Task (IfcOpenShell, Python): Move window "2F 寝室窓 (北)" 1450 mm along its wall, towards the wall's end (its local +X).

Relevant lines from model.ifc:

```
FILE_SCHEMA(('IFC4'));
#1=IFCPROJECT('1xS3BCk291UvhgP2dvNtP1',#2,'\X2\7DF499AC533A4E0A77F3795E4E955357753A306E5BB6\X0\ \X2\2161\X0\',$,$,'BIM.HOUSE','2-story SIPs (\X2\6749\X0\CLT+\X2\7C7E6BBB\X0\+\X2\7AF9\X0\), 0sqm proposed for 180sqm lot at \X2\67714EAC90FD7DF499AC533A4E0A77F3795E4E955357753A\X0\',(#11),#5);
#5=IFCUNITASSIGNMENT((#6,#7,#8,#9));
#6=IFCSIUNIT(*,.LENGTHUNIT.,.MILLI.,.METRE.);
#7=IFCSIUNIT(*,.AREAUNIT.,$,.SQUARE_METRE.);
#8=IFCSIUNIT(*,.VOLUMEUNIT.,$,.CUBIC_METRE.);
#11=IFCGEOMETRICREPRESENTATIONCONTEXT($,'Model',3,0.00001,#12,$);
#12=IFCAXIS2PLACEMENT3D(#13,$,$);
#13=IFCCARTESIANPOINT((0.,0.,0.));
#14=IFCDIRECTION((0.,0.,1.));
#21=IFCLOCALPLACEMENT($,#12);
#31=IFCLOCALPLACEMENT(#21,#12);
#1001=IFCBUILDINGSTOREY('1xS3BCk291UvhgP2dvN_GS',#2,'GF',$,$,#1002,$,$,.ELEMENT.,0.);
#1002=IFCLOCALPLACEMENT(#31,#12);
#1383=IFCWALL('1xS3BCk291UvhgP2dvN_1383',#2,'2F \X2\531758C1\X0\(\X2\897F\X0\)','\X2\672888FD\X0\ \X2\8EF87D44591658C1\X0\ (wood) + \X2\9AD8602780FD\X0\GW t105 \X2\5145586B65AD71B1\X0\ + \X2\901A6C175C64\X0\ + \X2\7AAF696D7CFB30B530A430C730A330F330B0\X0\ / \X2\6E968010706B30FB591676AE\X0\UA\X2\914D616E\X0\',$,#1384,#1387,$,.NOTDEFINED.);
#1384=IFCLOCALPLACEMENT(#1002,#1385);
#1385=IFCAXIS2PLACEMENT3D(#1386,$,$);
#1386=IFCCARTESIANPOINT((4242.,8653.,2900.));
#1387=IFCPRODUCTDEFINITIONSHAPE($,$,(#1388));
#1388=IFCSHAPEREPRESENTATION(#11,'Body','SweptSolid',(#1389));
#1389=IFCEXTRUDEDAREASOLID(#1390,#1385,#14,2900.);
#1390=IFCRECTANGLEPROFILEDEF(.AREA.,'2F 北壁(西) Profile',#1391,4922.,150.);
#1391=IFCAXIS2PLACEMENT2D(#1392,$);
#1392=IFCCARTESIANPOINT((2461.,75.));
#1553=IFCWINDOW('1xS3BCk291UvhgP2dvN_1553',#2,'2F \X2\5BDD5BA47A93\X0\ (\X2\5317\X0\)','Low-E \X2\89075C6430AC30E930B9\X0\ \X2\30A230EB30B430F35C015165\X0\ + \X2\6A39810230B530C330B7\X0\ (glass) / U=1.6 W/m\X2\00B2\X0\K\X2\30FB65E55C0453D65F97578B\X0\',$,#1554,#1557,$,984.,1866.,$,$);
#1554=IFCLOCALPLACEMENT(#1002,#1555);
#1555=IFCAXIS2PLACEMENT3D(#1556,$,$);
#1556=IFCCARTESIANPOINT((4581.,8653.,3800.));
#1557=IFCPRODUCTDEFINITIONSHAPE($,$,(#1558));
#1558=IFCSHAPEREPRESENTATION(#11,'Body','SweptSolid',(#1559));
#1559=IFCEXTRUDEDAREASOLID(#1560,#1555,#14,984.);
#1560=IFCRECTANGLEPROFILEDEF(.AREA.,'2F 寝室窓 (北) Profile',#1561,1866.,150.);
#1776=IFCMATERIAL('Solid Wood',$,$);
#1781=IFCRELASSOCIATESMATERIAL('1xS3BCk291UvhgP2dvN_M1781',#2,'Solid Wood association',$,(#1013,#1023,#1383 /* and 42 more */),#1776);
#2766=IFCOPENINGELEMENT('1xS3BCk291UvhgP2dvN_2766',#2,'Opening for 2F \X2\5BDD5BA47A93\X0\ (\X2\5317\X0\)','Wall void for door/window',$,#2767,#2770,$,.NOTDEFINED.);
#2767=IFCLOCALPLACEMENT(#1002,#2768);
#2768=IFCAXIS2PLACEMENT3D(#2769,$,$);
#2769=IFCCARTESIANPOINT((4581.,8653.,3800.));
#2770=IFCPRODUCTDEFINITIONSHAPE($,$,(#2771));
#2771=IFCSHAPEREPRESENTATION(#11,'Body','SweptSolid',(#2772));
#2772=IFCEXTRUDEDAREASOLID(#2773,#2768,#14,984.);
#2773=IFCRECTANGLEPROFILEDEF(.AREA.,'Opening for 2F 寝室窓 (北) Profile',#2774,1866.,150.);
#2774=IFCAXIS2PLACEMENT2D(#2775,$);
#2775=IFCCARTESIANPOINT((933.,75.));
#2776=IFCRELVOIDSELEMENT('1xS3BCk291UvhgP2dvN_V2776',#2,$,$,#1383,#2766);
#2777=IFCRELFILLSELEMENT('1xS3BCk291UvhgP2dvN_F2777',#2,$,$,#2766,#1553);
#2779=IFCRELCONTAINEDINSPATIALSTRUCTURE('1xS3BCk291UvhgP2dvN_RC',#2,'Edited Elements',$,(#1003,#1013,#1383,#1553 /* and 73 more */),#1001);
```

```python
import ifcopenshell
import ifcopenshell.api.geometry
import ifcopenshell.util.placement

model = ifcopenshell.open("model.ifc")

window = model.by_guid("1xS3BCk291UvhgP2dvN_1553")
opening = window.FillsVoids[0].RelatingOpeningElement
wall = opening.VoidsElements[0].RelatingBuildingElement

wall_matrix = ifcopenshell.util.placement.get_local_placement(wall.ObjectPlacement)
shift = wall_matrix[:3, 0] * 1450.0
before = ifcopenshell.util.placement.get_local_placement(window.ObjectPlacement)[:3, 3].copy()

# The window is not placed relative to its opening, so move both.
for product in (opening, window):
    matrix = ifcopenshell.util.placement.get_local_placement(product.ObjectPlacement)
    matrix[:3, 3] += shift
    ifcopenshell.api.geometry.edit_object_placement(model, product=product, matrix=matrix, is_si=False)

after = ifcopenshell.util.placement.get_local_placement(window.ObjectPlacement)[:3, 3]
print("window moved by", (after - before).round(3) + 0.0)

model.write("model-out.ifc")
```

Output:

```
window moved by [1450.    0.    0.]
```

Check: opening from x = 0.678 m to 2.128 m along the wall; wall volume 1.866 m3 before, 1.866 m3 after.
